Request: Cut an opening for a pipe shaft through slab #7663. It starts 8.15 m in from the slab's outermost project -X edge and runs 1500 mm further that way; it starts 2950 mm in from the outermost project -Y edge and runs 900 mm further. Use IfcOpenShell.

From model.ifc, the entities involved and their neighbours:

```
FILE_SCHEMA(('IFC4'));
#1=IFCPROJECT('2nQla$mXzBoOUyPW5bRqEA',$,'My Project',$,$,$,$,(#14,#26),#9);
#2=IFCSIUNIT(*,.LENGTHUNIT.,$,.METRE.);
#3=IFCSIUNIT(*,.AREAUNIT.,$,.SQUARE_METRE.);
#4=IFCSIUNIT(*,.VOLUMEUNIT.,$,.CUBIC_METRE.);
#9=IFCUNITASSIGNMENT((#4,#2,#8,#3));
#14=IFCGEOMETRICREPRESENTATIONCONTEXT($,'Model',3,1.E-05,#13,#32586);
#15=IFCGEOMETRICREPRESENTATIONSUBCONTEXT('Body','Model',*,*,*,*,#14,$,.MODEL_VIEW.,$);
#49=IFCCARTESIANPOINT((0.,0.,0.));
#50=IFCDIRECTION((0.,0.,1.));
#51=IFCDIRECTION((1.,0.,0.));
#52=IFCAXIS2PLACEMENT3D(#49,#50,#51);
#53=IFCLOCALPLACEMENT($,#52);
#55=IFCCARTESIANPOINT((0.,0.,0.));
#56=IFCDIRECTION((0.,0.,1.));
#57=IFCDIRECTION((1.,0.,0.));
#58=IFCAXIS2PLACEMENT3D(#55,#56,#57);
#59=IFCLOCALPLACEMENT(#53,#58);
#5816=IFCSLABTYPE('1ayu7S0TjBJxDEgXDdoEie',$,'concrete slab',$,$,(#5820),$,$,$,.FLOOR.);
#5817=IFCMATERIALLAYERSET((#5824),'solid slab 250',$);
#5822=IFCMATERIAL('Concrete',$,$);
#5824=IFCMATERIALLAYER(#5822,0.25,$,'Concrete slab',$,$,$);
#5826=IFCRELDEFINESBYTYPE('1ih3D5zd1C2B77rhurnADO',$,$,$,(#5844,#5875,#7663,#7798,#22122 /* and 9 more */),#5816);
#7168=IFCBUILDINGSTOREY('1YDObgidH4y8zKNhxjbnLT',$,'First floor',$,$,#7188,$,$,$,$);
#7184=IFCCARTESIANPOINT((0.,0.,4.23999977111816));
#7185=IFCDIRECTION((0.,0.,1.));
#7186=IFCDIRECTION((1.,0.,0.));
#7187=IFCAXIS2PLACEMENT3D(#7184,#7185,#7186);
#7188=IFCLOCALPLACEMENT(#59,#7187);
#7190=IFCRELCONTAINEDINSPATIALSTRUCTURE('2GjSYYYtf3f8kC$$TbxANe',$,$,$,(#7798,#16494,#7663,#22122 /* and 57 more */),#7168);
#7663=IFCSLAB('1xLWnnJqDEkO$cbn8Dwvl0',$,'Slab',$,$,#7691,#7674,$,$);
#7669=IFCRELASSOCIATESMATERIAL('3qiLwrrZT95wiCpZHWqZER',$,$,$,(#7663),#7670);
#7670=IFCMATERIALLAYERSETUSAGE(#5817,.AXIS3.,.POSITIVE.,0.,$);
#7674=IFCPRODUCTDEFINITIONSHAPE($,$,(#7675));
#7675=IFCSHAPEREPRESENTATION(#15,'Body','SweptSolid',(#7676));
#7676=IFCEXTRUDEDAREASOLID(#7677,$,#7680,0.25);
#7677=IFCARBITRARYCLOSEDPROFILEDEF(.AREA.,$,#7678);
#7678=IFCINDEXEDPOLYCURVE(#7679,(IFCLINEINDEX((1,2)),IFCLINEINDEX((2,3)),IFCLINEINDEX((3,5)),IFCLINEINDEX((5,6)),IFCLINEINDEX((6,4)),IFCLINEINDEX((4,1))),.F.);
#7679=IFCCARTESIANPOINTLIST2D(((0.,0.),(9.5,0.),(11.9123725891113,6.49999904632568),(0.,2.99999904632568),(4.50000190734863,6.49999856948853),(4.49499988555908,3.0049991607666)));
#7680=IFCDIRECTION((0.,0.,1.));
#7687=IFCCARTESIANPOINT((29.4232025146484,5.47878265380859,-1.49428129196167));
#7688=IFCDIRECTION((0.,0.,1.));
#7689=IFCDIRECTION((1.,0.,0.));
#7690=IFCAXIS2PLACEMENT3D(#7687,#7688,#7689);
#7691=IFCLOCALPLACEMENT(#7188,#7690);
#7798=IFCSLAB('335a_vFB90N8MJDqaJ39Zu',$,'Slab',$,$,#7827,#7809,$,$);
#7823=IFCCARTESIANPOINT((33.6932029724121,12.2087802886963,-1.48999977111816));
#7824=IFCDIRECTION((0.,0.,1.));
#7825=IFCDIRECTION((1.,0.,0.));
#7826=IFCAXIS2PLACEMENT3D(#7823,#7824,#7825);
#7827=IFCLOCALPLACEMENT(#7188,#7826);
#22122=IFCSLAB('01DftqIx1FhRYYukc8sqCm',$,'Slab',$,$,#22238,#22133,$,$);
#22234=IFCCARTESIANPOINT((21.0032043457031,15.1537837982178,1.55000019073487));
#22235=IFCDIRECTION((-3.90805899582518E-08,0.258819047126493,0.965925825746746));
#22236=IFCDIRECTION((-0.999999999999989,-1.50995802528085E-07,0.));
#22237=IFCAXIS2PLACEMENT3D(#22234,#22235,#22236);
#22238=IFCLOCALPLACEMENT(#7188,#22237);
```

```python
import numpy as np
import ifcopenshell
import ifcopenshell.api.feature
import ifcopenshell.api.geometry
import ifcopenshell.api.root
import ifcopenshell.geom
import ifcopenshell.util.placement
import ifcopenshell.util.representation
import ifcopenshell.util.shape
import ifcopenshell.util.unit

model = ifcopenshell.open("model.ifc")
unit_scale = ifcopenshell.util.unit.calculate_unit_scale(model)
settings = ifcopenshell.geom.settings()


def volume(element):
    """Net volume in cubic metres, openings subtracted."""
    shape = ifcopenshell.geom.create_shape(settings, element)
    return ifcopenshell.util.shape.get_volume(shape.geometry)


slab = model.by_guid("1xLWnnJqDEkO$cbn8Dwvl0")
before = volume(slab)

# Extent in the slab's own axes, in metres. The edges named are its -X and -Y sides.
slab_shape = ifcopenshell.geom.create_shape(settings, slab)
vertices = ifcopenshell.util.shape.get_vertices(slab_shape.geometry)
x_min, y_min, bottom = vertices.min(axis=0)
top = vertices[:, 2].max()

opening = ifcopenshell.api.root.create_entity(model, ifc_class="IfcOpeningElement", name="Pipe shaft opening", predefined_type="OPENING")
context = ifcopenshell.util.representation.get_context(model, "Model", "Body", "MODEL_VIEW")
width, depth = 1.5, 0.9
outline = [(0.0, 0.0), (width, 0.0), (width, depth), (0.0, depth), (0.0, 0.0)]
# Overshoot both faces by 50 mm so the cut is clean.
shape = ifcopenshell.api.geometry.add_slab_representation(
    model, context=context, depth=top - bottom + 0.1, polyline=outline
)
ifcopenshell.api.geometry.assign_representation(model, product=opening, representation=shape)

matrix = ifcopenshell.util.placement.get_local_placement(slab.ObjectPlacement)
matrix[:, 3] = matrix @ np.append(np.array([x_min + 8.15, y_min + 2.95, bottom - 0.05]) / unit_scale, 1.0)
ifcopenshell.api.geometry.edit_object_placement(model, product=opening, matrix=matrix, is_si=False)
ifcopenshell.api.feature.add_feature(model, feature=opening, element=slab)

after = volume(slab)

print(f"slab volume {before:.3f} -> {after:.3f} m3")

model.write("model-out.ifc")
```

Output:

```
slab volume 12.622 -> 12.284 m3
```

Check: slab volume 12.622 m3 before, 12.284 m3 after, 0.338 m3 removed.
